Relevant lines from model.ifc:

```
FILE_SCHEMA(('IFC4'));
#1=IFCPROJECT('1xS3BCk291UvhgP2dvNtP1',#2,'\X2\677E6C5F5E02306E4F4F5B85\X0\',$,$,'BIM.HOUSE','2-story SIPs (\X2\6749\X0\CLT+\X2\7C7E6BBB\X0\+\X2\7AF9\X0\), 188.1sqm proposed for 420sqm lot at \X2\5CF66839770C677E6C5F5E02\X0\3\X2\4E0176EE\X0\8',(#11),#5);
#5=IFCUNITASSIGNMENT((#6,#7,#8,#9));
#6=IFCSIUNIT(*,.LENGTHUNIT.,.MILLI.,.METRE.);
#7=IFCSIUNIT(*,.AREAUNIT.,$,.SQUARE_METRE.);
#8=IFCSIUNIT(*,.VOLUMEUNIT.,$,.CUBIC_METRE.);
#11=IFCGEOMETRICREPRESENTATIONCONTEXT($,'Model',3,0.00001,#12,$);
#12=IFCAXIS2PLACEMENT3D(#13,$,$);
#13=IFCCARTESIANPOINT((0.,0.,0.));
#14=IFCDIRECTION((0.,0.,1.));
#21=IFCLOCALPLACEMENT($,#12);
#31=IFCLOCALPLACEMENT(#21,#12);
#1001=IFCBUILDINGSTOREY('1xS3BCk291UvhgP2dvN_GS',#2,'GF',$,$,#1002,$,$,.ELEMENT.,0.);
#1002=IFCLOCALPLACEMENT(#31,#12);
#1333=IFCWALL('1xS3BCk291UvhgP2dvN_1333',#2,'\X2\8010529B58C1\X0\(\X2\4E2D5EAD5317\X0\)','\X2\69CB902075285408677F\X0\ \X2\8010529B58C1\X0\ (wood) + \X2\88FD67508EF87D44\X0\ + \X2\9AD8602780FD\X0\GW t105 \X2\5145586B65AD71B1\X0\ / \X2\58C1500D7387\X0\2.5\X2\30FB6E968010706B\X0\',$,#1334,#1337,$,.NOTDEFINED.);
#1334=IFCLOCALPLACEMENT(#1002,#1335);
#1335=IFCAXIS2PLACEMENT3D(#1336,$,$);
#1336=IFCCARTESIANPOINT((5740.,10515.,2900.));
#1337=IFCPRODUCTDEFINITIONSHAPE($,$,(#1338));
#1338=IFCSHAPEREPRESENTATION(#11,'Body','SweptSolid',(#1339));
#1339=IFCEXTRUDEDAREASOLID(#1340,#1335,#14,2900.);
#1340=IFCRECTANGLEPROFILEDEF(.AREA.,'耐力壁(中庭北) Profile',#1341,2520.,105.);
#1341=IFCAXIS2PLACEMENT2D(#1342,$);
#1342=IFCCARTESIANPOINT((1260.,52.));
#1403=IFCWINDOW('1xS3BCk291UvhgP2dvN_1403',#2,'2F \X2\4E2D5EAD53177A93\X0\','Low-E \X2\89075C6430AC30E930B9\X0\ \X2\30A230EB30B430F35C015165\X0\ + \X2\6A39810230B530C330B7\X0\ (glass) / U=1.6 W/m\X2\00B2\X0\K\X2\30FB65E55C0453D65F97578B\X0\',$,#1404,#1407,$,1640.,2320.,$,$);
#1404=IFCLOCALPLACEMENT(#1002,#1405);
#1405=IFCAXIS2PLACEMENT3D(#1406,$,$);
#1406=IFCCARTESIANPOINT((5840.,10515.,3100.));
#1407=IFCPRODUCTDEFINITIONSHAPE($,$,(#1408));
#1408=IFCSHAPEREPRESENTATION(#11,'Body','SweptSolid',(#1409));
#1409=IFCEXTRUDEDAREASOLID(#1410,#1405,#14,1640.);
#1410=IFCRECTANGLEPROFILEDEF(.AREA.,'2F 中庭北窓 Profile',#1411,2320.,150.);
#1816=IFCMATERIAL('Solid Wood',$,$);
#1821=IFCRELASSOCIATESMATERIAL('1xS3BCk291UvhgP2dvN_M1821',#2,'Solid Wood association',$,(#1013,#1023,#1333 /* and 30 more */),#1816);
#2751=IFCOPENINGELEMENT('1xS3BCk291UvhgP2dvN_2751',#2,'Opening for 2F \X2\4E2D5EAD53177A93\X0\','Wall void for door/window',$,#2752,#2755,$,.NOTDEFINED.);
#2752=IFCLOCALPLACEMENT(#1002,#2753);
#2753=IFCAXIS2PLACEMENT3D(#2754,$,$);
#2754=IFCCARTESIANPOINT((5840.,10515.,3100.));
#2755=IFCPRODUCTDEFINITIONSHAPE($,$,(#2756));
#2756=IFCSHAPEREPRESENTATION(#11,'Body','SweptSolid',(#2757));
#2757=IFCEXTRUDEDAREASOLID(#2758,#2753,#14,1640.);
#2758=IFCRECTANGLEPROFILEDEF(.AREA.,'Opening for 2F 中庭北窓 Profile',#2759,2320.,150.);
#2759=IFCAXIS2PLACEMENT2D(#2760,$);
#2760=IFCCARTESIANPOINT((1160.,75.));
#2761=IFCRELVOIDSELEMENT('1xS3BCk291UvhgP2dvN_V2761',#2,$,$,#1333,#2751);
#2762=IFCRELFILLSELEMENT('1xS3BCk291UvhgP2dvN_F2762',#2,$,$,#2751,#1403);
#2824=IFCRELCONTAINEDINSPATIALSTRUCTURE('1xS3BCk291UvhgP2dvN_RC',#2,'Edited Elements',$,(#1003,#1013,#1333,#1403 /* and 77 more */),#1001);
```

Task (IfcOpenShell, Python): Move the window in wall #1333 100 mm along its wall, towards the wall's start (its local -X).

```python
import ifcopenshell
import ifcopenshell.api.geometry
import ifcopenshell.util.placement
import ifcopenshell.util.unit

model = ifcopenshell.open("model.ifc")
unit_scale = ifcopenshell.util.unit.calculate_unit_scale(model)

window = model.by_guid("1xS3BCk291UvhgP2dvN_1403")
opening = window.FillsVoids[0].RelatingOpeningElement
wall = opening.VoidsElements[0].RelatingBuildingElement

wall_matrix = ifcopenshell.util.placement.get_local_placement(wall.ObjectPlacement)
shift = wall_matrix[:3, 0] * -0.1 / unit_scale
before = ifcopenshell.util.placement.get_local_placement(window.ObjectPlacement)[:3, 3].copy()

# The window is not placed relative to its opening, so move both.
for product in (opening, window):
    matrix = ifcopenshell.util.placement.get_local_placement(product.ObjectPlacement)
    matrix[:3, 3] += shift
    ifcopenshell.api.geometry.edit_object_placement(model, product=product, matrix=matrix, is_si=False)

after = ifcopenshell.util.placement.get_local_placement(window.ObjectPlacement)[:3, 3]
print("window moved by", (after - before).round(3) + 0.0)

model.write("model-out.ifc")
```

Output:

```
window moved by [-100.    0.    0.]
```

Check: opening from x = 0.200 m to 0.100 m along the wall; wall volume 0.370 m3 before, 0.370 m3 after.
